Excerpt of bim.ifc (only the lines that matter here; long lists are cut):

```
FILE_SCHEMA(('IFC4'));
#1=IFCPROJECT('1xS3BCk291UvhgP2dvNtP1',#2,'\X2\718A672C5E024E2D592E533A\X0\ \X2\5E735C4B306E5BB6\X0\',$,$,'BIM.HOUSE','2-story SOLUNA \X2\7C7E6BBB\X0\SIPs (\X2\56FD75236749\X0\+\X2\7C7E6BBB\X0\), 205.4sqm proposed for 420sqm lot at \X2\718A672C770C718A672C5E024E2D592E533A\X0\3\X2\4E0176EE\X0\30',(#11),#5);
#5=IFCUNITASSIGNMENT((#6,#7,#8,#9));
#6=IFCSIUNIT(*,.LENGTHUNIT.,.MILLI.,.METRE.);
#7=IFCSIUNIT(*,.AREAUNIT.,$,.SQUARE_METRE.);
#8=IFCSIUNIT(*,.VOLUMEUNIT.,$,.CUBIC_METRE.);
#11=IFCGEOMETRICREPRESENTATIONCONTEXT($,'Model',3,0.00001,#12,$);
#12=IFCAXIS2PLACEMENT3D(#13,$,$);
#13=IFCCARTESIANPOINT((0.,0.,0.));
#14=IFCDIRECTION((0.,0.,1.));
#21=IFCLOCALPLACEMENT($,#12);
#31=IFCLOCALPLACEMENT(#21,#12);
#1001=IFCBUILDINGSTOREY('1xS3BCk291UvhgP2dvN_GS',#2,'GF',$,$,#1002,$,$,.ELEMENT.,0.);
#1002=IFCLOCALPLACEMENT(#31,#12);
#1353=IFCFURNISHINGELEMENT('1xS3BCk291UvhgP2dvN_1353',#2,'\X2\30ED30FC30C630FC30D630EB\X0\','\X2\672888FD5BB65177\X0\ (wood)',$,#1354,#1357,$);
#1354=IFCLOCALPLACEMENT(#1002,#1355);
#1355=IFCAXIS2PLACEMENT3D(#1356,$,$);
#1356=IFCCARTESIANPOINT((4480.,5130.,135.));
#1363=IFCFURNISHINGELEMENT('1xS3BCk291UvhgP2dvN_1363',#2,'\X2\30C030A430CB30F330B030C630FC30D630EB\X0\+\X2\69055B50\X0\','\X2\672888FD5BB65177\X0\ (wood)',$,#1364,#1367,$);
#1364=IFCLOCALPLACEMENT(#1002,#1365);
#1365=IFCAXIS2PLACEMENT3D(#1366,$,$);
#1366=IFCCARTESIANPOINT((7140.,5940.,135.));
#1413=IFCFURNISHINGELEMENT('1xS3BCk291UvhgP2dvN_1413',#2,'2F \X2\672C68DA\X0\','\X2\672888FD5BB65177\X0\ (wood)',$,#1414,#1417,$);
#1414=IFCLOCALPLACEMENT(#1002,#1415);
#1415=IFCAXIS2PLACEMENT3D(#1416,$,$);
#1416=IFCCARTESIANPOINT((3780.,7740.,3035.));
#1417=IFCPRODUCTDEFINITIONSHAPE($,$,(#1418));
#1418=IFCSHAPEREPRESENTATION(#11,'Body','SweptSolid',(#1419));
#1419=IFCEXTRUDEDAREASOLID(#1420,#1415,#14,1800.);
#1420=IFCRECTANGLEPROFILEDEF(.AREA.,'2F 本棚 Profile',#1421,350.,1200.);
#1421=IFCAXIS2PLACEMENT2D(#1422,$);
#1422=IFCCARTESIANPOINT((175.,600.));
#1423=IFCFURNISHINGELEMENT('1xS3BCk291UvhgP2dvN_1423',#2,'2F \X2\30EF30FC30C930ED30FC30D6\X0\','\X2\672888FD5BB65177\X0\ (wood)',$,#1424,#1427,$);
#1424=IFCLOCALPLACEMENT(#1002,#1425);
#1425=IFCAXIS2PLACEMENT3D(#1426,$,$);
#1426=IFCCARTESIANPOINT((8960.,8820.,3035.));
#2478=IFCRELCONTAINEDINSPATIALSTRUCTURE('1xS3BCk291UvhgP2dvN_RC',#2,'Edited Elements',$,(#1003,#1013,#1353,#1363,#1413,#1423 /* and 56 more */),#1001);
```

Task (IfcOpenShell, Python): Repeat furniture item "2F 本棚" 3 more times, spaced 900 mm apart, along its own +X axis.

```python
import ifcopenshell
import ifcopenshell.api.geometry
import ifcopenshell.api.root
import ifcopenshell.util.element
import ifcopenshell.util.placement

model = ifcopenshell.open("bim.ifc")


def reuse_history(source, copy):
    """copy_class also copies each property set's owner history, people and application; keep the originals."""
    for rel in copy.IsDefinedBy:
        if rel.is_a("IfcRelDefinesByProperties") and (history := rel.RelatingPropertyDefinition.OwnerHistory):
            rel.RelatingPropertyDefinition.OwnerHistory = source.OwnerHistory
            ifcopenshell.util.element.remove_deep2(model, history)


source = model.by_guid("1xS3BCk291UvhgP2dvN_1413")
base = ifcopenshell.util.placement.get_local_placement(source.ObjectPlacement)
step = base[:3, 0] * 900.0

for i in range(1, 4):
    copy = ifcopenshell.api.root.copy_class(model, product=source)
    copy.Representation = ifcopenshell.util.element.copy_deep(
        model, source.Representation, exclude=["IfcGeometricRepresentationContext", "IfcRepresentationMap"]
    )
    reuse_history(source, copy)
    matrix = base.copy()
    matrix[:3, 3] += i * step
    print("added at", matrix[:3, 3].round(3) + 0.0)
    ifcopenshell.api.geometry.edit_object_placement(model, product=copy, matrix=matrix, is_si=False)

model.write("bim_v2.ifc")
```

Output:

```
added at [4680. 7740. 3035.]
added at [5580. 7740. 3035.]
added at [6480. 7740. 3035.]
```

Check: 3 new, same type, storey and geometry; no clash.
